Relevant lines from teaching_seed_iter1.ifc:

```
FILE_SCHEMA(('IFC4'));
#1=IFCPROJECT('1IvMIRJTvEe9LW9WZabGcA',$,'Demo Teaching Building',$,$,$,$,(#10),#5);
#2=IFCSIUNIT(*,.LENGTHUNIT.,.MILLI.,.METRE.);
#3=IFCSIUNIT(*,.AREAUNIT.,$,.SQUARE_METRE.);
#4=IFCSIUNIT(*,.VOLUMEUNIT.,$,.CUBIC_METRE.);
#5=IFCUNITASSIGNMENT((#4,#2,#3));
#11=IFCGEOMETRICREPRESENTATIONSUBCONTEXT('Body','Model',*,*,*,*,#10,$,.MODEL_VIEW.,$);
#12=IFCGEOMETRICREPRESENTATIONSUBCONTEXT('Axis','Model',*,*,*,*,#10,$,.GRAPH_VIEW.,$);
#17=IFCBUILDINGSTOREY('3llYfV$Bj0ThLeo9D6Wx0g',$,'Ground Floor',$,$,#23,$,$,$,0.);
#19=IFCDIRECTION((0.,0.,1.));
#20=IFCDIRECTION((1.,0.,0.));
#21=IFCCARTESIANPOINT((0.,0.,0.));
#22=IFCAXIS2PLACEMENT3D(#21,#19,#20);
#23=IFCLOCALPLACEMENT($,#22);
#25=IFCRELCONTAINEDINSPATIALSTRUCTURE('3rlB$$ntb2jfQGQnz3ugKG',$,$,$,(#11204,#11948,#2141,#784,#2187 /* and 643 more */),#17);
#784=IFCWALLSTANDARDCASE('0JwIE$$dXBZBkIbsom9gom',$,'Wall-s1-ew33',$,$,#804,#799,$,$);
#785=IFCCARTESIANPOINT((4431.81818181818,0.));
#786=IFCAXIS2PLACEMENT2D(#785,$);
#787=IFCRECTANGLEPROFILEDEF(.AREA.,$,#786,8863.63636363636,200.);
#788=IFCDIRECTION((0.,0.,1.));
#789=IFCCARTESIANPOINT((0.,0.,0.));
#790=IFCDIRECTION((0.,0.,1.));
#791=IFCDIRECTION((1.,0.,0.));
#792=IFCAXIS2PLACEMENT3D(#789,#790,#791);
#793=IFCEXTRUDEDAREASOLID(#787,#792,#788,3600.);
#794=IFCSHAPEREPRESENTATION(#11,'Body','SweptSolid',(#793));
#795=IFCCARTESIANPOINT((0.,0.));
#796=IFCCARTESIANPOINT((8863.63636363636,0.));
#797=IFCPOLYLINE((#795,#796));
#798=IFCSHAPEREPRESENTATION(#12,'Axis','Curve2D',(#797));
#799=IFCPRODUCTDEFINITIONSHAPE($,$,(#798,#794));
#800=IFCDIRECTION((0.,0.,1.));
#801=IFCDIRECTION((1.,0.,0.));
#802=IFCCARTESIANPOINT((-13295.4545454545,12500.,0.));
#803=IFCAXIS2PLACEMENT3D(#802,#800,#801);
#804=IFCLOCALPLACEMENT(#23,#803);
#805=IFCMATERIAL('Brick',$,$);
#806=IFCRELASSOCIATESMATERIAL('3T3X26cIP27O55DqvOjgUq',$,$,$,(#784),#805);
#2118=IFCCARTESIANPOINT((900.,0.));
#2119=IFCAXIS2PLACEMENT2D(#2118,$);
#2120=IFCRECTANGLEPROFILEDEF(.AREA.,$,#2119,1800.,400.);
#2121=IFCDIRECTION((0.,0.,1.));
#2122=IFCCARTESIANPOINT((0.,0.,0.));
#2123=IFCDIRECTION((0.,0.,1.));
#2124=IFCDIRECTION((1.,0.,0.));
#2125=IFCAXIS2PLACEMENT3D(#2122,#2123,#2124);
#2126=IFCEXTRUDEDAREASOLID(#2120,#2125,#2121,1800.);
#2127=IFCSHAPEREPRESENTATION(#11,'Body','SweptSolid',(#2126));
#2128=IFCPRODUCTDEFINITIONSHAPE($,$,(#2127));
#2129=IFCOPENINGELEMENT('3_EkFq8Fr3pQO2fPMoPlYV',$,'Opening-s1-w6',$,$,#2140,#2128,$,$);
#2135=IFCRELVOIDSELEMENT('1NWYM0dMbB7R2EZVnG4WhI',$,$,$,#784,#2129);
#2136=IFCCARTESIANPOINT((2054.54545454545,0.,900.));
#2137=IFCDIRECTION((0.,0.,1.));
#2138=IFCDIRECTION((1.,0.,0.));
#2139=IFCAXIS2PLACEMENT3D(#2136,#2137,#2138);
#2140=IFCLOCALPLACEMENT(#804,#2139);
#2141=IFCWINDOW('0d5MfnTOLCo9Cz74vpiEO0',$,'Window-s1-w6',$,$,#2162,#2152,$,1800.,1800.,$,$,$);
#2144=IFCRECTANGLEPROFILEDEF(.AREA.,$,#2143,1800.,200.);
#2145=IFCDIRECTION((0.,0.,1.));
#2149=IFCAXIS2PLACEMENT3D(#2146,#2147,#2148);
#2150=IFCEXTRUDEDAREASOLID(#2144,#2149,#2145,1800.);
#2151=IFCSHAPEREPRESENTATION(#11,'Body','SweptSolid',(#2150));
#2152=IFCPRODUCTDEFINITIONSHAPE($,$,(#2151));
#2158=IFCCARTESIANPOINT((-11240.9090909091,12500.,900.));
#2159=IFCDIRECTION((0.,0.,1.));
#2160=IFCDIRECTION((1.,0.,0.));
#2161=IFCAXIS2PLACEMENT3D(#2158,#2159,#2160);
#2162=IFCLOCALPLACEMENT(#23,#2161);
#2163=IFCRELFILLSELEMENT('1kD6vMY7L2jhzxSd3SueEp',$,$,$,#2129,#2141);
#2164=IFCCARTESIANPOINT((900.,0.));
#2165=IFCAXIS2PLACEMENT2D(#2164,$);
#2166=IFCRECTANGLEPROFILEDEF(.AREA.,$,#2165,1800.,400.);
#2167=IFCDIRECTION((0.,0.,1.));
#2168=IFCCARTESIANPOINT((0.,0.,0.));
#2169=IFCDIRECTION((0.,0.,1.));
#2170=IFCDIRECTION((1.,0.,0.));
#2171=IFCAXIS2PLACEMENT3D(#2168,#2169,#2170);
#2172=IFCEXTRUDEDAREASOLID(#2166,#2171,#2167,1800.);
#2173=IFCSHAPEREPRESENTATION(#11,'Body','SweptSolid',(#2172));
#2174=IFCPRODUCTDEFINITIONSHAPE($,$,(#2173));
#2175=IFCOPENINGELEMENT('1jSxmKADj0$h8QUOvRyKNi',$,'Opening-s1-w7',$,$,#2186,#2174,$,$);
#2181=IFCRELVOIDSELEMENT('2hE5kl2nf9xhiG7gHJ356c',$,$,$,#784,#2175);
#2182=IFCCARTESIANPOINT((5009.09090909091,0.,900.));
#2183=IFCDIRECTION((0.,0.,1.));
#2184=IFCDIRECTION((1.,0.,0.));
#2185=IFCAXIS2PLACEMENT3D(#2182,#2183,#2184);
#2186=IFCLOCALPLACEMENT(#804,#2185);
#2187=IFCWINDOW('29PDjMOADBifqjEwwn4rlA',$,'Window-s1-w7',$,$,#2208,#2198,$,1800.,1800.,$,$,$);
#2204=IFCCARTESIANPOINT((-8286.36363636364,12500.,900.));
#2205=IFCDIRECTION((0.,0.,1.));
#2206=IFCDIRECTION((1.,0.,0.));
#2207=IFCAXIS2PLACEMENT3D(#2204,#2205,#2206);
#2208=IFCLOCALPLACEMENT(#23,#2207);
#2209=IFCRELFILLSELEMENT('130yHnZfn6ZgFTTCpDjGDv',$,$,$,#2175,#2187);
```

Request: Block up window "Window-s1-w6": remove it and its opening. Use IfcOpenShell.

```python
import ifcopenshell
import ifcopenshell.api.feature
import ifcopenshell.api.root
import ifcopenshell.geom
import ifcopenshell.util.shape

model = ifcopenshell.open("teaching_seed_iter1.ifc")
settings = ifcopenshell.geom.settings()


def volume(element):
    """Net volume in cubic metres, openings subtracted."""
    shape = ifcopenshell.geom.create_shape(settings, element)
    return ifcopenshell.util.shape.get_volume(shape.geometry)


window = model.by_guid("0d5MfnTOLCo9Cz74vpiEO0")
opening = window.FillsVoids[0].RelatingOpeningElement
wall = opening.VoidsElements[0].RelatingBuildingElement
before = volume(wall)

ifcopenshell.api.root.remove_product(model, product=window)
ifcopenshell.api.feature.remove_feature(model, feature=opening)

after = volume(wall)

print(f"wall volume {before:.3f} -> {after:.3f} m3")

model.write("teaching_seed_iter1_rev.ifc")
```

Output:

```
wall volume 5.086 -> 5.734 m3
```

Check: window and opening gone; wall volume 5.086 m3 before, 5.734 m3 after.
